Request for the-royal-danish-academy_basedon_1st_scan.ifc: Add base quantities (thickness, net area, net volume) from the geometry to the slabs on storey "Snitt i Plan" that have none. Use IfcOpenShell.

First a look at what the model holds.

```python
import ifcopenshell
import ifcopenshell.util.element
import ifcopenshell.util.unit

model = ifcopenshell.open("the-royal-danish-academy_basedon_1st_scan.ifc")
print(model.schema)
for unit_type in ("LENGTHUNIT", "AREAUNIT", "VOLUMEUNIT"):
    print(unit_type, ifcopenshell.util.unit.calculate_unit_scale(model, unit_type))
storey = next(s for s in model.by_type("IfcBuildingStorey") if s.Name == "Snitt i Plan")
slabs = [e for e in ifcopenshell.util.element.get_decomposition(storey) if e.is_a("IfcSlab")]
for e in sorted(slabs, key=lambda e: e.id()):
    print(e.id(), e.is_a(), e.Name, list(ifcopenshell.util.element.get_psets(e, qtos_only=True)), sep=" | ")
```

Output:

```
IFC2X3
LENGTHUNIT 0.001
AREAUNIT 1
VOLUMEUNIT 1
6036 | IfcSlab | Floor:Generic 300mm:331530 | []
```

```python
import ifcopenshell
import ifcopenshell.api.pset
import ifcopenshell.geom
import ifcopenshell.util.element
import ifcopenshell.util.shape
import ifcopenshell.util.unit

model = ifcopenshell.open("the-royal-danish-academy_basedon_1st_scan.ifc")
unit_scale = ifcopenshell.util.unit.calculate_unit_scale(model)
area_scale = ifcopenshell.util.unit.calculate_unit_scale(model, "AREAUNIT")
volume_scale = ifcopenshell.util.unit.calculate_unit_scale(model, "VOLUMEUNIT")
settings = ifcopenshell.geom.settings()

storey = next(s for s in model.by_type("IfcBuildingStorey") if s.Name == "Snitt i Plan")
slabs = [e for e in ifcopenshell.util.element.get_decomposition(storey) if e.is_a("IfcSlab")]

for e in sorted(slabs, key=lambda e: e.id()):
    if ifcopenshell.util.element.get_psets(e, qtos_only=True, should_inherit=False):
        continue
    # Geometry comes back in metres, in the element's own axes.
    shape = ifcopenshell.geom.create_shape(settings, e)
    values = {
        "Width": ifcopenshell.util.shape.get_z(shape.geometry) / unit_scale,
        "NetArea": ifcopenshell.util.shape.get_footprint_area(shape.geometry) / area_scale,
        "NetVolume": ifcopenshell.util.shape.get_volume(shape.geometry) / volume_scale,
    }
    qto = ifcopenshell.api.pset.add_qto(model, product=e, name="BaseQuantities")
    ifcopenshell.api.pset.edit_qto(model, qto=qto, properties=values)
    print(e.id(), {k: round(v, 3) for k, v in values.items()})

model.write("the-royal-danish-academy_basedon_1st_scan_updated.ifc")
```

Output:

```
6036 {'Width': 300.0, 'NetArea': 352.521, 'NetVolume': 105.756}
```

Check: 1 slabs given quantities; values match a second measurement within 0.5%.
